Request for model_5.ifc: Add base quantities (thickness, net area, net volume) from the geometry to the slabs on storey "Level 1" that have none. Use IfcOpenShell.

First a look at what the model holds.

```python
import ifcopenshell
import ifcopenshell.util.element
import ifcopenshell.util.unit

model = ifcopenshell.open("model_5.ifc")
print(model.schema)
for unit_type in ("LENGTHUNIT", "AREAUNIT", "VOLUMEUNIT"):
    print(unit_type, ifcopenshell.util.unit.calculate_unit_scale(model, unit_type))
storey = next(s for s in model.by_type("IfcBuildingStorey") if s.Name == "Level 1")
slabs = [e for e in ifcopenshell.util.element.get_decomposition(storey) if e.is_a("IfcSlab")]
for e in sorted(slabs, key=lambda e: e.id()):
    print(e.id(), e.is_a(), e.Name, list(ifcopenshell.util.element.get_psets(e, qtos_only=True)), sep=" | ")
```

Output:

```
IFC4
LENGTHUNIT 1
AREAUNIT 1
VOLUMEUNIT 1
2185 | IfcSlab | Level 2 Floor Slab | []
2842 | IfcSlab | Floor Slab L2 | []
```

```python
import ifcopenshell
import ifcopenshell.api.pset
import ifcopenshell.geom
import ifcopenshell.util.element
import ifcopenshell.util.shape
import ifcopenshell.util.unit

model = ifcopenshell.open("model_5.ifc")
unit_scale = ifcopenshell.util.unit.calculate_unit_scale(model)
area_scale = ifcopenshell.util.unit.calculate_unit_scale(model, "AREAUNIT")
volume_scale = ifcopenshell.util.unit.calculate_unit_scale(model, "VOLUMEUNIT")
settings = ifcopenshell.geom.settings()

storey = next(s for s in model.by_type("IfcBuildingStorey") if s.Name == "Level 1")
slabs = [e for e in ifcopenshell.util.element.get_decomposition(storey) if e.is_a("IfcSlab")]

for e in sorted(slabs, key=lambda e: e.id()):
    if ifcopenshell.util.element.get_psets(e, qtos_only=True, should_inherit=False):
        continue
    # Geometry comes back in metres, in the element's own axes.
    shape = ifcopenshell.geom.create_shape(settings, e)
    values = {
        "Width": ifcopenshell.util.shape.get_z(shape.geometry) / unit_scale,
        "NetArea": ifcopenshell.util.shape.get_footprint_area(shape.geometry) / area_scale,
        "NetVolume": ifcopenshell.util.shape.get_volume(shape.geometry) / volume_scale,
    }
    qto = ifcopenshell.api.pset.add_qto(model, product=e, name="Qto_SlabBaseQuantities")
    ifcopenshell.api.pset.edit_qto(model, qto=qto, properties=values)
    print(e.id(), {k: round(v, 3) for k, v in values.items()})

model.write("model_5-out.ifc")
```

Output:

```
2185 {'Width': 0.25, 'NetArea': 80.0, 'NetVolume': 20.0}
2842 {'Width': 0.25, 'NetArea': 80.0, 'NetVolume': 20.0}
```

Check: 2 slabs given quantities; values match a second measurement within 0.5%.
